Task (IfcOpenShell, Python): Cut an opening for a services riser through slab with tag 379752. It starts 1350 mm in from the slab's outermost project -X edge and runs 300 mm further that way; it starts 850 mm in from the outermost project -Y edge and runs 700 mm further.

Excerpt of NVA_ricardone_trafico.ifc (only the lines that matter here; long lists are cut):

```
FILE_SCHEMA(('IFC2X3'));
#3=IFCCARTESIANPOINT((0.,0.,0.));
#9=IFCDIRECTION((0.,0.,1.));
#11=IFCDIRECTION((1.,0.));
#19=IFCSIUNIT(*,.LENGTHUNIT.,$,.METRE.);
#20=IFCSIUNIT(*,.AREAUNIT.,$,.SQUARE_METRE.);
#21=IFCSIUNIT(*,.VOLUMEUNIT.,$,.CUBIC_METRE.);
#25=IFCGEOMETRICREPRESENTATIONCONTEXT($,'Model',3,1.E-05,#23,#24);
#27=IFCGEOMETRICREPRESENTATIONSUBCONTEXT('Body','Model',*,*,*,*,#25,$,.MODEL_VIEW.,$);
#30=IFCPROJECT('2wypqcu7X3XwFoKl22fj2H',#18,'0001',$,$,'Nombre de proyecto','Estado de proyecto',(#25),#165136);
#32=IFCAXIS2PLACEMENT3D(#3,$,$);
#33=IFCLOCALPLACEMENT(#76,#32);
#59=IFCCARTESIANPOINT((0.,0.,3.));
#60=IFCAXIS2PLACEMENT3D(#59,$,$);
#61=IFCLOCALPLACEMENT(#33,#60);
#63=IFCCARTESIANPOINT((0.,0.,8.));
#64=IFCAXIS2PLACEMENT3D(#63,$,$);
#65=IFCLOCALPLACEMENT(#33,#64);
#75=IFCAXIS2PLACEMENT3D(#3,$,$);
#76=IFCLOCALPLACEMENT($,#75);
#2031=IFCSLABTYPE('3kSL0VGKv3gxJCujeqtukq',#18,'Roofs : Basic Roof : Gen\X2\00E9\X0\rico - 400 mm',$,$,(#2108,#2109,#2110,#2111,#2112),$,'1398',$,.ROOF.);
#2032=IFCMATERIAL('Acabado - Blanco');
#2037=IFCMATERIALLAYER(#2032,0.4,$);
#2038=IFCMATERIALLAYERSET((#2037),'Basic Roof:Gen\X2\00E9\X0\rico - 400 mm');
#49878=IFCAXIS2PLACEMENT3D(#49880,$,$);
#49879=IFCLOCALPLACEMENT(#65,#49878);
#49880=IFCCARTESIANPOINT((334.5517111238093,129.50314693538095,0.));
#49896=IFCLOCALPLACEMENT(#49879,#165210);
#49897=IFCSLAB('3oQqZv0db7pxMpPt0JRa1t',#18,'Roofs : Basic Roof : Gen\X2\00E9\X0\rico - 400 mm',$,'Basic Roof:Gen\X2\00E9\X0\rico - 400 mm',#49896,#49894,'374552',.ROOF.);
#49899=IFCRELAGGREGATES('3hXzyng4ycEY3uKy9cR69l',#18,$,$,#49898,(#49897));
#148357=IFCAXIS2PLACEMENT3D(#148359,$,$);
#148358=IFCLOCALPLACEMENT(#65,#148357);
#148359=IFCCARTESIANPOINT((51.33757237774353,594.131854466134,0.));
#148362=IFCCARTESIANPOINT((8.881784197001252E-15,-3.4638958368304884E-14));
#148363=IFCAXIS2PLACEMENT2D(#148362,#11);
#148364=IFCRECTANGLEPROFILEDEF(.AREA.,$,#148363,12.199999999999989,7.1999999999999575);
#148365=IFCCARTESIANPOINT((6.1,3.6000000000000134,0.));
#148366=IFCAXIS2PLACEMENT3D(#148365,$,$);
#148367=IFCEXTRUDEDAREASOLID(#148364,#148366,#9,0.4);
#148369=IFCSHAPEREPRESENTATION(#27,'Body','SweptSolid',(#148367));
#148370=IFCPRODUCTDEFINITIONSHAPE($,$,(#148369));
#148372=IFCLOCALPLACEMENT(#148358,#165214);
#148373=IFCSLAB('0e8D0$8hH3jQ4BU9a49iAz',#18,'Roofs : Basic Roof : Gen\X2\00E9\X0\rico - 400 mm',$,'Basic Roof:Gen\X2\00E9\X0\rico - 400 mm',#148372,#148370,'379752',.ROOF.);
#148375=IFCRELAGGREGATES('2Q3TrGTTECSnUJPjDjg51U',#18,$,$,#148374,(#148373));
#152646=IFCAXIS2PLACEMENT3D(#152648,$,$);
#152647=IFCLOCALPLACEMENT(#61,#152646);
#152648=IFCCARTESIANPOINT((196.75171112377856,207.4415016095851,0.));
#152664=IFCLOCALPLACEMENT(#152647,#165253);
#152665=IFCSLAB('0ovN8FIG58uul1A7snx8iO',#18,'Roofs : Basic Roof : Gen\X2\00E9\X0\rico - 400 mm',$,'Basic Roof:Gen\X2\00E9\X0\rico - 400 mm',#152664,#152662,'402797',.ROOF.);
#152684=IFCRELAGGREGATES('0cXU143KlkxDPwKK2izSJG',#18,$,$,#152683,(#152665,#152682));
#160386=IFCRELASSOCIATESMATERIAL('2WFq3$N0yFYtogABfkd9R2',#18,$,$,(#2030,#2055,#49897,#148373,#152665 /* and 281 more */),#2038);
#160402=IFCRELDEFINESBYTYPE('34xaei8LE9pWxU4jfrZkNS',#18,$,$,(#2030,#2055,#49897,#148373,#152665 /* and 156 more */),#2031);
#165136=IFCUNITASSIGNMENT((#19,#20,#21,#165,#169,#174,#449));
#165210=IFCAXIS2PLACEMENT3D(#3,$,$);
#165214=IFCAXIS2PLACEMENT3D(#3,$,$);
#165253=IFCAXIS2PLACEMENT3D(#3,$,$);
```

```python
import numpy as np
import ifcopenshell
import ifcopenshell.api.feature
import ifcopenshell.api.geometry
import ifcopenshell.api.root
import ifcopenshell.geom
import ifcopenshell.util.placement
import ifcopenshell.util.representation
import ifcopenshell.util.shape
import ifcopenshell.util.unit

model = ifcopenshell.open("NVA_ricardone_trafico.ifc")
unit_scale = ifcopenshell.util.unit.calculate_unit_scale(model)
settings = ifcopenshell.geom.settings()


def volume(element):
    """Net volume in cubic metres, openings subtracted."""
    shape = ifcopenshell.geom.create_shape(settings, element)
    return ifcopenshell.util.shape.get_volume(shape.geometry)


slab = model.by_guid("0e8D0$8hH3jQ4BU9a49iAz")
before = volume(slab)

# Extent in the slab's own axes, in metres. The edges named are its -X and -Y sides.
slab_shape = ifcopenshell.geom.create_shape(settings, slab)
vertices = ifcopenshell.util.shape.get_vertices(slab_shape.geometry)
x_min, y_min, bottom = vertices.min(axis=0)
top = vertices[:, 2].max()

opening = ifcopenshell.api.root.create_entity(model, ifc_class="IfcOpeningElement", name="Services riser opening")
context = ifcopenshell.util.representation.get_context(model, "Model", "Body", "MODEL_VIEW")
width, depth = 0.3, 0.7
outline = [(0.0, 0.0), (width, 0.0), (width, depth), (0.0, depth), (0.0, 0.0)]
# Overshoot both faces by 50 mm so the cut is clean.
shape = ifcopenshell.api.geometry.add_slab_representation(
    model, context=context, depth=top - bottom + 0.1, polyline=outline
)
ifcopenshell.api.geometry.assign_representation(model, product=opening, representation=shape)

matrix = ifcopenshell.util.placement.get_local_placement(slab.ObjectPlacement)
matrix[:, 3] = matrix @ np.append(np.array([x_min + 1.35, y_min + 0.85, bottom - 0.05]) / unit_scale, 1.0)
ifcopenshell.api.geometry.edit_object_placement(model, product=opening, matrix=matrix, is_si=False)
ifcopenshell.api.feature.add_feature(model, feature=opening, element=slab)

after = volume(slab)

print(f"slab volume {before:.3f} -> {after:.3f} m3")

model.write("NVA_ricardone_trafico_v2.ifc")
```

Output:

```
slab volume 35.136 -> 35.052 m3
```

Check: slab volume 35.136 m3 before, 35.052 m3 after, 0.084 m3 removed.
